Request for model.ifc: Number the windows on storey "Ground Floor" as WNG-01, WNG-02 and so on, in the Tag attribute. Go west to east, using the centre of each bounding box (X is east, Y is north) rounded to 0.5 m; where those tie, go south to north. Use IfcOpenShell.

First a look at what the model holds.

```python
import ifcopenshell
import ifcopenshell.util.element
import ifcopenshell.util.placement

model = ifcopenshell.open("model.ifc")
print(model.schema)
storey = next(s for s in model.by_type("IfcBuildingStorey") if s.Name == "Ground Floor")
windows = [e for e in ifcopenshell.util.element.get_decomposition(storey) if e.is_a("IfcWindow")]
for e in sorted(windows, key=lambda e: e.id()):
    origin = ifcopenshell.util.placement.get_local_placement(e.ObjectPlacement)[:3, 3]
    print(e.id(), e.Tag, e.Name, origin.round(2) + 0.0, sep=" | ")
```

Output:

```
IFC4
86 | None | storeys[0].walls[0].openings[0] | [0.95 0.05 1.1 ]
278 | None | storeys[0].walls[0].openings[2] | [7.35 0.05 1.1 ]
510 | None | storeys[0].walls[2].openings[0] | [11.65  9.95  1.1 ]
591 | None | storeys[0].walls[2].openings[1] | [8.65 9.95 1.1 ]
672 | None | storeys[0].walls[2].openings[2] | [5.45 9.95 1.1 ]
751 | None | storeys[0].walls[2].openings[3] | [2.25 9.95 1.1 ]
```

```python
import ifcopenshell
import ifcopenshell.geom
import ifcopenshell.util.element
import ifcopenshell.util.shape

model = ifcopenshell.open("model.ifc")
settings = ifcopenshell.geom.settings()
settings.set("use-world-coords", True)


def centre(element):
    shape = ifcopenshell.geom.create_shape(settings, element)
    return ifcopenshell.util.shape.get_bbox_centroid(shape.geometry)


storey = next(s for s in model.by_type("IfcBuildingStorey") if s.Name == "Ground Floor")
windows = [e for e in ifcopenshell.util.element.get_decomposition(storey) if e.is_a("IfcWindow")]

# Insertion points can sit at a corner or the storey origin, so sort by the geometry (in metres).
centres = {e: centre(e) for e in windows}
windows.sort(key=lambda e: (round(centres[e][0] / 0.5), centres[e][1]))

for i, e in enumerate(windows, start=1):
    number = f"WNG-{i:02d}"
    e.Tag = number
    print(e.id(), number)

model.write("model_updated.ifc")
```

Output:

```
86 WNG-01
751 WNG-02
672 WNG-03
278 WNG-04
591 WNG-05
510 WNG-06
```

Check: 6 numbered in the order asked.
